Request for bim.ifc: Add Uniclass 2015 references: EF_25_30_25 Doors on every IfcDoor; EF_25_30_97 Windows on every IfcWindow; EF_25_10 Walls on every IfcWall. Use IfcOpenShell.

First a look at what the model holds.

```python
import ifcopenshell

model = ifcopenshell.open("bim.ifc")
print(model.schema)
print("classifications:", [c.Name for c in model.by_type("IfcClassification")])
for ifc_class in ("IfcDoor", "IfcRoof", "IfcStair", "IfcWall", "IfcWindow"):
    print(ifc_class, len(model.by_type(ifc_class)))
```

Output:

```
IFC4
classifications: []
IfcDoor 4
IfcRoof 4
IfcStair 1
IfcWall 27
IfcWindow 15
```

```python
import ifcopenshell
import ifcopenshell.api.classification

model = ifcopenshell.open("bim.ifc")

system = ifcopenshell.api.classification.add_classification(model, classification="Uniclass 2015")

codes = {
    "IfcDoor": ("EF_25_30_25", "Doors"),
    "IfcWindow": ("EF_25_30_97", "Windows"),
    "IfcWall": ("EF_25_10", "Walls"),
}
for ifc_class, (code, name) in codes.items():
    products = model.by_type(ifc_class)
    ifcopenshell.api.classification.add_reference(
        model, products=products, classification=system, identification=code, name=name
    )
    print(code, len(products))

model.write("bim_rev.ifc")
```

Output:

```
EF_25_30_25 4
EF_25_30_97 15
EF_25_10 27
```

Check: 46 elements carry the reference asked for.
